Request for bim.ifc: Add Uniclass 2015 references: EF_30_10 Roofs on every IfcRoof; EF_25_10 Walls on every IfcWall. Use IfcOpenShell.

First a look at what the model holds.

```python
import ifcopenshell

model = ifcopenshell.open("bim.ifc")
print(model.schema)
print("classifications:", [c.Name for c in model.by_type("IfcClassification")])
for ifc_class in ("IfcDoor", "IfcRoof", "IfcStair", "IfcWall", "IfcWindow"):
    print(ifc_class, len(model.by_type(ifc_class)))
```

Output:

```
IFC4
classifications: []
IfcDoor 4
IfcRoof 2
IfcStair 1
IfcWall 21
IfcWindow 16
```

```python
import ifcopenshell
import ifcopenshell.api.classification

model = ifcopenshell.open("bim.ifc")

system = ifcopenshell.api.classification.add_classification(model, classification="Uniclass 2015")

codes = {
    "IfcRoof": ("EF_30_10", "Roofs"),
    "IfcWall": ("EF_25_10", "Walls"),
}
for ifc_class, (code, name) in codes.items():
    products = model.by_type(ifc_class)
    ifcopenshell.api.classification.add_reference(
        model, products=products, classification=system, identification=code, name=name
    )
    print(code, len(products))

model.write("bim-out.ifc")
```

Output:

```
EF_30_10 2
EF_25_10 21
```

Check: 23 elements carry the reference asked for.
